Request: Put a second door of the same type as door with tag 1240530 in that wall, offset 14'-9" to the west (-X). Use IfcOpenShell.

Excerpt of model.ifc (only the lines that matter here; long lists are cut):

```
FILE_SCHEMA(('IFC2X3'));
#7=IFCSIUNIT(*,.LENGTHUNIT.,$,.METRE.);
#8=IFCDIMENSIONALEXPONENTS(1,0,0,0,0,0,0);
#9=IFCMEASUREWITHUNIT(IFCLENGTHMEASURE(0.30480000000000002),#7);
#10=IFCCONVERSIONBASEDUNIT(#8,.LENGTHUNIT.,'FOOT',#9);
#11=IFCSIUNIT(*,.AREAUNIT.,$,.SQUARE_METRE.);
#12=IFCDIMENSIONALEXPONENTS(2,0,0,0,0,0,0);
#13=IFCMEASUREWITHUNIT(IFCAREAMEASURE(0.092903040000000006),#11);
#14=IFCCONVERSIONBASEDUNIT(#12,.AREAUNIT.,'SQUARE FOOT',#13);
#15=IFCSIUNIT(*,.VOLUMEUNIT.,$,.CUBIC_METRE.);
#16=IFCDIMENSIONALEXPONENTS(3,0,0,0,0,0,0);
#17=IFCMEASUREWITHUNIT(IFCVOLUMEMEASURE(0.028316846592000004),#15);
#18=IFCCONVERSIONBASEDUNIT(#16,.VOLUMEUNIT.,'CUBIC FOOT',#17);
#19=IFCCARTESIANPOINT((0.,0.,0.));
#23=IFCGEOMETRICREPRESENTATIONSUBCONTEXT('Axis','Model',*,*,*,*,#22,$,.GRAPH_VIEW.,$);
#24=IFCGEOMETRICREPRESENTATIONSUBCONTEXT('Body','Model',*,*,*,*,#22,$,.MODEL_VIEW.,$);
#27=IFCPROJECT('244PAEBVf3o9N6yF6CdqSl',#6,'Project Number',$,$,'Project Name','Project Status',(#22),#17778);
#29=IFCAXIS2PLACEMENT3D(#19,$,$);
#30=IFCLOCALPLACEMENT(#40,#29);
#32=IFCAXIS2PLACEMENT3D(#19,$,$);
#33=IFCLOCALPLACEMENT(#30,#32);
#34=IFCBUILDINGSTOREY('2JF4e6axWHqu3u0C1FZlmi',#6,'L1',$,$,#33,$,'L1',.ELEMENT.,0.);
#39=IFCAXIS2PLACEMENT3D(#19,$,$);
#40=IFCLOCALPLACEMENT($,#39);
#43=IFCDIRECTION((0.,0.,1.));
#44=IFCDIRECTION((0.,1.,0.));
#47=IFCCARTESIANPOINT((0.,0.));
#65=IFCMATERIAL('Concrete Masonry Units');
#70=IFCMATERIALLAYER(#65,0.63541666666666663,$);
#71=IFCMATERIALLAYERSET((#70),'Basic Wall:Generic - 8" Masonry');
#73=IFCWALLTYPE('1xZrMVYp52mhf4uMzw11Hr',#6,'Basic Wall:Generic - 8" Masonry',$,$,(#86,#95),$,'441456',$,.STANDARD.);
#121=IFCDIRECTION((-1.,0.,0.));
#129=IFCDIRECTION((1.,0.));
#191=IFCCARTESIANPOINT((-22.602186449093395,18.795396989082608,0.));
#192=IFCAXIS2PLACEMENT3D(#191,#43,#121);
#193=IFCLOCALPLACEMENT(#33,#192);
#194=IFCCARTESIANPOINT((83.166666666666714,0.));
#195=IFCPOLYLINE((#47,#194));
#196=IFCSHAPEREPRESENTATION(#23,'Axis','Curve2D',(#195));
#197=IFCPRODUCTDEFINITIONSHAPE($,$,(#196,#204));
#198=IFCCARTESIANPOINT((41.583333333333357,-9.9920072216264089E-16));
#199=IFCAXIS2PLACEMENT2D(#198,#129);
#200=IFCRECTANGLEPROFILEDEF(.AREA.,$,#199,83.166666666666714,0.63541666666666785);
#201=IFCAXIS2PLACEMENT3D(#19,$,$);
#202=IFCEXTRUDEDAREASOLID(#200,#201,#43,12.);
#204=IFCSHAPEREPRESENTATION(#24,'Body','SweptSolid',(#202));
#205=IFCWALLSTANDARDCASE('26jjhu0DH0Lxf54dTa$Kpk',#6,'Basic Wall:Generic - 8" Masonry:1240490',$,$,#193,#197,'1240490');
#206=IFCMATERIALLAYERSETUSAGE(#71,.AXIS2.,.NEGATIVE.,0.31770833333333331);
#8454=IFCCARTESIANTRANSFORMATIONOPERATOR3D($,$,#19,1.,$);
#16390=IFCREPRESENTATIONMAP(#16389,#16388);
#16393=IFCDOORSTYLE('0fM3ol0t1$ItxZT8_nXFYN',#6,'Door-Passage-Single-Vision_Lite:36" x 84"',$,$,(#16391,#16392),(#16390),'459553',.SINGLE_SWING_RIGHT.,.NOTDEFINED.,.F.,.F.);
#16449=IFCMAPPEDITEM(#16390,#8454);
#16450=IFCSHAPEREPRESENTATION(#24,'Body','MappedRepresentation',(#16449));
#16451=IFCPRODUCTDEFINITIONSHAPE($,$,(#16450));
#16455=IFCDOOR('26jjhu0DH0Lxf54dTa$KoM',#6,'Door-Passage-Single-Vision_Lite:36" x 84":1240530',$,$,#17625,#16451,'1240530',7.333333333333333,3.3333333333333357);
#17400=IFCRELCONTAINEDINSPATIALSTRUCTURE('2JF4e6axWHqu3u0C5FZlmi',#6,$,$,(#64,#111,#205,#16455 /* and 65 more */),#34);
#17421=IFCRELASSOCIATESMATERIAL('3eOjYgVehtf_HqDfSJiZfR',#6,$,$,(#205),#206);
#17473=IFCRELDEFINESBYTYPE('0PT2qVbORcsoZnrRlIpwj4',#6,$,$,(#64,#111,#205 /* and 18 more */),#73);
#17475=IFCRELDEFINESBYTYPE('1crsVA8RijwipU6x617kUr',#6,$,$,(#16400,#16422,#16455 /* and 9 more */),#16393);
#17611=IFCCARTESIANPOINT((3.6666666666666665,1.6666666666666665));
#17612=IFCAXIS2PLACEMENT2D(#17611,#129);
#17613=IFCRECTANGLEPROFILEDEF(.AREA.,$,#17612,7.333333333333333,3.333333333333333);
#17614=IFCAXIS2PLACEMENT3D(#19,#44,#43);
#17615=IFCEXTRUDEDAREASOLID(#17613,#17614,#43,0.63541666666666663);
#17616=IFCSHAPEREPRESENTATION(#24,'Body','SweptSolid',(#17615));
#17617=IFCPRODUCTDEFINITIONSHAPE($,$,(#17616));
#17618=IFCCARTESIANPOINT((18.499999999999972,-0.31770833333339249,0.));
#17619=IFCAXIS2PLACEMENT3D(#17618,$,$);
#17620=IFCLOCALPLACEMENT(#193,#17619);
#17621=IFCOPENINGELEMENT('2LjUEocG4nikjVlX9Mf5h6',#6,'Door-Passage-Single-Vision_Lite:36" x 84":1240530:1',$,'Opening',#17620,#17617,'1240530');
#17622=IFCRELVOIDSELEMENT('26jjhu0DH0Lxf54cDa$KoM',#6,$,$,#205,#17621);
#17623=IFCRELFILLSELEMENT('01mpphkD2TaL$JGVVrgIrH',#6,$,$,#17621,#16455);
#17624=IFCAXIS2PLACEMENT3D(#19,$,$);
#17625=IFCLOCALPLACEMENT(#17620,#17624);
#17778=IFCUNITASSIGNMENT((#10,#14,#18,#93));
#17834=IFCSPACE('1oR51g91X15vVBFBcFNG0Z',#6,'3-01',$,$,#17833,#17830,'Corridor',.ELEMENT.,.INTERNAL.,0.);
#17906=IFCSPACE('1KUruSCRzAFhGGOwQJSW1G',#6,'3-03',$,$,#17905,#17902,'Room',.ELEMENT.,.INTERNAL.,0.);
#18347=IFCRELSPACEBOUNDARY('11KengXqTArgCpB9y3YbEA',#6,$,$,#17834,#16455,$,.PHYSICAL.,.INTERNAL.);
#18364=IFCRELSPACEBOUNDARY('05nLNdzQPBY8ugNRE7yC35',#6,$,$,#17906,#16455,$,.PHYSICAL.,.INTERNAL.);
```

```python
import ifcopenshell
import ifcopenshell.api.feature
import ifcopenshell.api.geometry
import ifcopenshell.api.root
import ifcopenshell.geom
import ifcopenshell.util.element
import ifcopenshell.util.placement
import ifcopenshell.util.shape
import ifcopenshell.util.unit

model = ifcopenshell.open("model.ifc")
unit_scale = ifcopenshell.util.unit.calculate_unit_scale(model)
settings = ifcopenshell.geom.settings()


def volume(element):
    """Net volume in cubic metres, openings subtracted."""
    shape = ifcopenshell.geom.create_shape(settings, element)
    return ifcopenshell.util.shape.get_volume(shape.geometry)


def reuse_history(source, copy):
    """copy_class also copies each property set's owner history, people and application; keep the originals."""
    for rel in copy.IsDefinedBy:
        if rel.is_a("IfcRelDefinesByProperties") and (history := rel.RelatingPropertyDefinition.OwnerHistory):
            rel.RelatingPropertyDefinition.OwnerHistory = source.OwnerHistory
            ifcopenshell.util.element.remove_deep2(model, history)


door = model.by_guid("26jjhu0DH0Lxf54dTa$KoM")
opening = door.FillsVoids[0].RelatingOpeningElement
wall = opening.VoidsElements[0].RelatingBuildingElement
before = volume(wall)
shift = ifcopenshell.util.placement.get_local_placement(wall.ObjectPlacement)[:3, 0] * 177 * 0.0254 / unit_scale

# copy_class copies the void relationship, type, container and properties, but no geometry.
new_opening = ifcopenshell.api.root.copy_class(model, product=opening)
new_opening.Representation = ifcopenshell.util.element.copy_deep(
    model, opening.Representation, exclude=["IfcGeometricRepresentationContext", "IfcRepresentationMap"]
)
new_opening.Name = 'Door-Passage-Single-Vision_Lite:36" x 84"'
new_opening.Tag = None
new_door = ifcopenshell.api.root.copy_class(model, product=door)
new_door.Representation = ifcopenshell.util.element.copy_deep(
    model, door.Representation, exclude=["IfcGeometricRepresentationContext", "IfcRepresentationMap"]
)
new_door.Name = 'Door-Passage-Single-Vision_Lite:36" x 84"'
new_door.Tag = None
reuse_history(door, new_door)
fills = ifcopenshell.api.feature.add_filling(model, opening=new_opening, element=new_door)
fills.OwnerHistory = new_door.OwnerHistory  # required in IFC2X3

for old, new in ((opening, new_opening), (door, new_door)):
    matrix = ifcopenshell.util.placement.get_local_placement(old.ObjectPlacement)
    matrix[:3, 3] += shift
    ifcopenshell.api.geometry.edit_object_placement(model, product=new, matrix=matrix, is_si=False)

after = volume(wall)

print(f"wall volume {before:.3f} -> {after:.3f} m3")

model.write("model_edited.ifc")
```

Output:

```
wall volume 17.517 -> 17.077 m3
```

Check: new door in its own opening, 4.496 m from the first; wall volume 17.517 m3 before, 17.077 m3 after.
